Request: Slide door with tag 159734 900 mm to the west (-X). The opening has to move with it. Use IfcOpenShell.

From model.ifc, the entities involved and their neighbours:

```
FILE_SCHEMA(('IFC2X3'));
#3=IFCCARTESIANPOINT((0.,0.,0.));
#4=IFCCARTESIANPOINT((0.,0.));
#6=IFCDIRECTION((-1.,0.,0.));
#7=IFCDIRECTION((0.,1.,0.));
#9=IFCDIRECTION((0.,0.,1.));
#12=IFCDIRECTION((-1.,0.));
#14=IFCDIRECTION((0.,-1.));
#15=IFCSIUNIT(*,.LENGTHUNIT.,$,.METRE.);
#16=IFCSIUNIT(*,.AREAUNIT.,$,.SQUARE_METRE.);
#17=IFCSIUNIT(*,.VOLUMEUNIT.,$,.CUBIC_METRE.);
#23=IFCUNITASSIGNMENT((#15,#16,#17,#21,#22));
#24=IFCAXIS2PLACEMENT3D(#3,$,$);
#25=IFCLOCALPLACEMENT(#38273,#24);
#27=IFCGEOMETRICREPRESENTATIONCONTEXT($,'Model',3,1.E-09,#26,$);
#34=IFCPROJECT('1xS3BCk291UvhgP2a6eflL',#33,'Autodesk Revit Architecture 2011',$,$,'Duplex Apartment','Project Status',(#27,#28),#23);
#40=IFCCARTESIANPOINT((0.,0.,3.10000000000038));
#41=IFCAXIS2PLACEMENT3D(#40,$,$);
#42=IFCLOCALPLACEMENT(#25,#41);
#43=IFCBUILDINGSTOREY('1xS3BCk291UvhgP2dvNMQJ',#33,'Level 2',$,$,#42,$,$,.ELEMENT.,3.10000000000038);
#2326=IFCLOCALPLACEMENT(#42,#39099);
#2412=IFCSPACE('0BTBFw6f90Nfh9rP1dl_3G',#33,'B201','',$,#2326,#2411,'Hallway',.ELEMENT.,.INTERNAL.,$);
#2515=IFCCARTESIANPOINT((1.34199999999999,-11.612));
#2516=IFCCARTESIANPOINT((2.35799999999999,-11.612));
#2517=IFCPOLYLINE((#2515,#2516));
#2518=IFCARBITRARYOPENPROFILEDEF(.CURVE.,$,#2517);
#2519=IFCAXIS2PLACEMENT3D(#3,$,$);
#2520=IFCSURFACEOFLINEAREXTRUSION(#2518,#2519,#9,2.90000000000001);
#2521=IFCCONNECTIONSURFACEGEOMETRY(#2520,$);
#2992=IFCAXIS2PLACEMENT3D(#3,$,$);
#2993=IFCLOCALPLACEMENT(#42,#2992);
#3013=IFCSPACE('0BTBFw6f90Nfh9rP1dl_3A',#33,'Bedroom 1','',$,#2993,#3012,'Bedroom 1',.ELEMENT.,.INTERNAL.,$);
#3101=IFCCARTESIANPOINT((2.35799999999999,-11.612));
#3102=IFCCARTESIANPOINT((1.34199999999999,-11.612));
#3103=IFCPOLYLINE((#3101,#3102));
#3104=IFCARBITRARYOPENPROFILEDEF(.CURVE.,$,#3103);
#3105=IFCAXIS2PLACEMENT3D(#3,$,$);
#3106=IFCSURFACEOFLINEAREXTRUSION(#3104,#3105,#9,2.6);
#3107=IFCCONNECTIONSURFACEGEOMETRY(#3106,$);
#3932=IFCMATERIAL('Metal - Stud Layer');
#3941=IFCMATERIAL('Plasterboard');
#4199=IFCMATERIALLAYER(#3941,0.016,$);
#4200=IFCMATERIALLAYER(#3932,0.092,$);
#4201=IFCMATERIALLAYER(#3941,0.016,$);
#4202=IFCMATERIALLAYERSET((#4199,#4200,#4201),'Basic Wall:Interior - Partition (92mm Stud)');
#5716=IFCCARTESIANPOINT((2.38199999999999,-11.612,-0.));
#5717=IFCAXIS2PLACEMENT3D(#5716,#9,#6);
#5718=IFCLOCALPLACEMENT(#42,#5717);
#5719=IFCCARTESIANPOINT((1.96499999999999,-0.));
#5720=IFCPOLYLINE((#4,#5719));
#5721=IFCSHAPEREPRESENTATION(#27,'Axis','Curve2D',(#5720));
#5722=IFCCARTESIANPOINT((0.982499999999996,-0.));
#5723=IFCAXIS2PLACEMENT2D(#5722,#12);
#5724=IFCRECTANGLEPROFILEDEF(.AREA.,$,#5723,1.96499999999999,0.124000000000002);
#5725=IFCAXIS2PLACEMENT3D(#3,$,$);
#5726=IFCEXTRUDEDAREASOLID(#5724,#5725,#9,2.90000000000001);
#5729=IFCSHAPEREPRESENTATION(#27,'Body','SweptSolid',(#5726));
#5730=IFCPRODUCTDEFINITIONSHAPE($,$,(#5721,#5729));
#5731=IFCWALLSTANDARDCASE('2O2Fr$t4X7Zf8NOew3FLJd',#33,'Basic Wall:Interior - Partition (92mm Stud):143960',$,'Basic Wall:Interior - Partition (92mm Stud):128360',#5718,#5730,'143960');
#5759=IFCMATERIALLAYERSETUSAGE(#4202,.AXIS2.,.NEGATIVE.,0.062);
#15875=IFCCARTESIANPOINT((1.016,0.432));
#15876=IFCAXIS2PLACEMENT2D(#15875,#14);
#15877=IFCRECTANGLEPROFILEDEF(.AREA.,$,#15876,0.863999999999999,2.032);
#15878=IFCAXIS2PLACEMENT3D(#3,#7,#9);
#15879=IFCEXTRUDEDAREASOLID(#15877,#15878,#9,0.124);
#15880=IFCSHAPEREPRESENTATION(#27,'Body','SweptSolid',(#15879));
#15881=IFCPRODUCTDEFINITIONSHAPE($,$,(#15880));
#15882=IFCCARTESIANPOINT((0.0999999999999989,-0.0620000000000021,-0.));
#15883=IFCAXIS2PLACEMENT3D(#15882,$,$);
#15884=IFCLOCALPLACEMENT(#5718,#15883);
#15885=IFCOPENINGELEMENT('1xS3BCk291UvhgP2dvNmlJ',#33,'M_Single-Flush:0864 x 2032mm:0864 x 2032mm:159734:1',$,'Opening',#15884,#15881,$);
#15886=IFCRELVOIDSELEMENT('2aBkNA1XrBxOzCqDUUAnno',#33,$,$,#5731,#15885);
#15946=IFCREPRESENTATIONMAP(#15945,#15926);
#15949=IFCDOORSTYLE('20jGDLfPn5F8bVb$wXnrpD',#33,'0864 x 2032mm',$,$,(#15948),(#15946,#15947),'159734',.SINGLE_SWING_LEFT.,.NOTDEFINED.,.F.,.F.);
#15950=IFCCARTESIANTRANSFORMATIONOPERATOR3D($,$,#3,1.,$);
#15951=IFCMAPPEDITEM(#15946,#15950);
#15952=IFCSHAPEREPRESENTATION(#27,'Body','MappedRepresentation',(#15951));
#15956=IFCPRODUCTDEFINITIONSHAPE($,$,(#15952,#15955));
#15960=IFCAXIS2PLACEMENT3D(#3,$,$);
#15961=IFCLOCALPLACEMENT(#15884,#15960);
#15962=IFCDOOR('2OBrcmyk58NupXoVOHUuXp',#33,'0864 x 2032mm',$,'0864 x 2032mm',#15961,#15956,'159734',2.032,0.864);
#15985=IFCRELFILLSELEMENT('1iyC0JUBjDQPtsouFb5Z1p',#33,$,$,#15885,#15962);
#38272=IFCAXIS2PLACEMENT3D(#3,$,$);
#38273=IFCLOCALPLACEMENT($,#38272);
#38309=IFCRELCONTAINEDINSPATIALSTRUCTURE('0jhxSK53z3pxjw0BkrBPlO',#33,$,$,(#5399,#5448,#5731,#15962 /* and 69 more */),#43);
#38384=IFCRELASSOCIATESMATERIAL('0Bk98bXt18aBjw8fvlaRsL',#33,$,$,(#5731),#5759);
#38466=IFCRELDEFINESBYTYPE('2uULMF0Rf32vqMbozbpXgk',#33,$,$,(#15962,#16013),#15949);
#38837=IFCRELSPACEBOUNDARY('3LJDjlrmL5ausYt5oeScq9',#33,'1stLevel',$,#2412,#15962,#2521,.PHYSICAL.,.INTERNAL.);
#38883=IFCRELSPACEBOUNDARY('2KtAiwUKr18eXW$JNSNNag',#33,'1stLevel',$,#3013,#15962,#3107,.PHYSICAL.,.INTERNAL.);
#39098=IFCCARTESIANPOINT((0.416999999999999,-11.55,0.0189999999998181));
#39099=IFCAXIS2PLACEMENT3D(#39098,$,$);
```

```python
import numpy as np
import ifcopenshell
import ifcopenshell.api.geometry
import ifcopenshell.util.placement
import ifcopenshell.util.unit

model = ifcopenshell.open("model.ifc")
unit_scale = ifcopenshell.util.unit.calculate_unit_scale(model)

door = model.by_guid("2OBrcmyk58NupXoVOHUuXp")
opening = door.FillsVoids[0].RelatingOpeningElement
wall = opening.VoidsElements[0].RelatingBuildingElement

wall_matrix = ifcopenshell.util.placement.get_local_placement(wall.ObjectPlacement)
shift = wall_matrix[:3, 0] * 0.9 / unit_scale
before = ifcopenshell.util.placement.get_local_placement(door.ObjectPlacement)[:3, 3].copy()

# The door is placed relative to its opening, so it follows when the opening moves.
matrix = ifcopenshell.util.placement.get_local_placement(opening.ObjectPlacement)
matrix[:3, 3] += shift
ifcopenshell.api.geometry.edit_object_placement(
    model, product=opening, matrix=matrix, is_si=False, should_transform_children=True
)

# Space boundary surfaces are stored in each space's coordinates; move them too.
for rel in door.ProvidesBoundaries:
    if not rel.ConnectionGeometry:
        continue
    surface = rel.ConnectionGeometry.SurfaceOnRelatingElement
    space_matrix = ifcopenshell.util.placement.get_local_placement(rel.RelatingSpace.ObjectPlacement)
    point = np.array(surface.Position.Location.Coordinates) + space_matrix[:3, :3].T @ shift
    surface.Position = model.createIfcAxis2Placement3D(
        model.createIfcCartesianPoint(point.tolist()), surface.Position.Axis, surface.Position.RefDirection
    )

after = ifcopenshell.util.placement.get_local_placement(door.ObjectPlacement)[:3, 3]
print("door moved by", (after - before).round(3) + 0.0)

model.write("model_v2.ifc")
```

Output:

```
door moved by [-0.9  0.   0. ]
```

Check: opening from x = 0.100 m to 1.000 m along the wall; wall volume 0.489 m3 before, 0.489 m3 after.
